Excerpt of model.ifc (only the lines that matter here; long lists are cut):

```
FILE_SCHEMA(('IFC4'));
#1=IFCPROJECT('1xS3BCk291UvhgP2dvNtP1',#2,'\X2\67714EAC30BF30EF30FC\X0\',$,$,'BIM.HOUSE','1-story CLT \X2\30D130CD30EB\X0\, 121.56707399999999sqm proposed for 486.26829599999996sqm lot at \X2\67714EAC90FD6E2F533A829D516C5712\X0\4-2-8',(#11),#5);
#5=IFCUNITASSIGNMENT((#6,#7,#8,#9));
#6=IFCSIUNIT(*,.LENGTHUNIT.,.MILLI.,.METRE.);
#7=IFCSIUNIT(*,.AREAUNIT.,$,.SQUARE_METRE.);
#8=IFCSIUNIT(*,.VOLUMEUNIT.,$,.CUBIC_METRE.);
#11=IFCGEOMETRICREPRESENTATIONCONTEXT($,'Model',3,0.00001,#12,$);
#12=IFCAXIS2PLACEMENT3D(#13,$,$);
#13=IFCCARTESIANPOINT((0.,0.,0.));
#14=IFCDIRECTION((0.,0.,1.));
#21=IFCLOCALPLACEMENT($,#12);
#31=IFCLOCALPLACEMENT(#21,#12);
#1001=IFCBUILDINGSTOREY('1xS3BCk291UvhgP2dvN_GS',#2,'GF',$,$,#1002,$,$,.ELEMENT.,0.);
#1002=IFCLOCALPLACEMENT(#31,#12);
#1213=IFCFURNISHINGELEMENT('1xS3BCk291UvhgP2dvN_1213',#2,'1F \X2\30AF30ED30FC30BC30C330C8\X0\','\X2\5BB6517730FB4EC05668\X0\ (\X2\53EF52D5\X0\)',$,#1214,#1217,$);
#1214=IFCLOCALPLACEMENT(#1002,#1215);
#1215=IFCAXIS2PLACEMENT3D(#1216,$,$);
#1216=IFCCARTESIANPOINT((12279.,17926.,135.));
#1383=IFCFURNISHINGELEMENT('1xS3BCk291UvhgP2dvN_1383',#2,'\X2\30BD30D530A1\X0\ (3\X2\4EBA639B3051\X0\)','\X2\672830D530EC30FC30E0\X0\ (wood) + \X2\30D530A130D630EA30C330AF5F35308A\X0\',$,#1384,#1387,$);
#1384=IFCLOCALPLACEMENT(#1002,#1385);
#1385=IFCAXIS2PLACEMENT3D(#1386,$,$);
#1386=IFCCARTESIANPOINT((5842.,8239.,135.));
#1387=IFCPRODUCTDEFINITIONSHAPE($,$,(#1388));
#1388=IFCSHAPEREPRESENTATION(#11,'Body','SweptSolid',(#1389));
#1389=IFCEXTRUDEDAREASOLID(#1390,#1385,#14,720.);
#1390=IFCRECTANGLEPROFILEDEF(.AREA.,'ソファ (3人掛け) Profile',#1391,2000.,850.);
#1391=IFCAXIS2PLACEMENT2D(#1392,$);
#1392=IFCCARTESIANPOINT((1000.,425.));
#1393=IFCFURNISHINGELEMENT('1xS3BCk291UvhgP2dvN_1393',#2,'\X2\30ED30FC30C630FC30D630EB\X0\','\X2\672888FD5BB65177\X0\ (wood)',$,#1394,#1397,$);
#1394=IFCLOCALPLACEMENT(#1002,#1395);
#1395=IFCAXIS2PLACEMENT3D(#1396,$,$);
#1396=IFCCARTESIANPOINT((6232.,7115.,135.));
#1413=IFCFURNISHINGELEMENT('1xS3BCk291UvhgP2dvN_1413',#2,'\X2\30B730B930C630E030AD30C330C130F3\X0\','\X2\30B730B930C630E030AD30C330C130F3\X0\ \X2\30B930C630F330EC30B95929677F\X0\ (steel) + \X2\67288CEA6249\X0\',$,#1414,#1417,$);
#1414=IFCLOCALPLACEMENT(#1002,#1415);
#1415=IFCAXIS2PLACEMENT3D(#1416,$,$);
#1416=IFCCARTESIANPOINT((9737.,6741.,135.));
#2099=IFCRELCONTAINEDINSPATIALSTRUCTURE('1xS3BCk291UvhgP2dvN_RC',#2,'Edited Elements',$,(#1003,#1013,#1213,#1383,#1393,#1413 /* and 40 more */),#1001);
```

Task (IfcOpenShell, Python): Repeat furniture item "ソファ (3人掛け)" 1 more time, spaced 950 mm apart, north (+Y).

```python
import numpy as np
import ifcopenshell
import ifcopenshell.api.geometry
import ifcopenshell.api.root
import ifcopenshell.util.element
import ifcopenshell.util.placement

model = ifcopenshell.open("model.ifc")


def reuse_history(source, copy):
    """copy_class also copies each property set's owner history, people and application; keep the originals."""
    for rel in copy.IsDefinedBy:
        if rel.is_a("IfcRelDefinesByProperties") and (history := rel.RelatingPropertyDefinition.OwnerHistory):
            rel.RelatingPropertyDefinition.OwnerHistory = source.OwnerHistory
            ifcopenshell.util.element.remove_deep2(model, history)


source = model.by_guid("1xS3BCk291UvhgP2dvN_1383")
base = ifcopenshell.util.placement.get_local_placement(source.ObjectPlacement)
step = np.array([0.0, 1.0, 0.0]) * 950.0

for i in range(1, 2):
    copy = ifcopenshell.api.root.copy_class(model, product=source)
    copy.Representation = ifcopenshell.util.element.copy_deep(
        model, source.Representation, exclude=["IfcGeometricRepresentationContext", "IfcRepresentationMap"]
    )
    reuse_history(source, copy)
    matrix = base.copy()
    matrix[:3, 3] += i * step
    print("added at", matrix[:3, 3].round(3) + 0.0)
    ifcopenshell.api.geometry.edit_object_placement(model, product=copy, matrix=matrix, is_si=False)

model.write("model_edited.ifc")
```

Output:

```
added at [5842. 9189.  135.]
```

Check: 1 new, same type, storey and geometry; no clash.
